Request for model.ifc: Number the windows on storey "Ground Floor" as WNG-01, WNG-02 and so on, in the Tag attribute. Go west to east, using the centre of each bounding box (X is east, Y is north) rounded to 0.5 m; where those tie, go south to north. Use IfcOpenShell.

First a look at what the model holds.

```python
import ifcopenshell
import ifcopenshell.util.element
import ifcopenshell.util.placement

model = ifcopenshell.open("model.ifc")
print(model.schema)
storey = next(s for s in model.by_type("IfcBuildingStorey") if s.Name == "Ground Floor")
windows = [e for e in ifcopenshell.util.element.get_decomposition(storey) if e.is_a("IfcWindow")]
for e in sorted(windows, key=lambda e: e.id()):
    origin = ifcopenshell.util.placement.get_local_placement(e.ObjectPlacement)[:3, 3]
    print(e.id(), e.Tag, e.Name, origin.round(2) + 0.0, sep=" | ")
```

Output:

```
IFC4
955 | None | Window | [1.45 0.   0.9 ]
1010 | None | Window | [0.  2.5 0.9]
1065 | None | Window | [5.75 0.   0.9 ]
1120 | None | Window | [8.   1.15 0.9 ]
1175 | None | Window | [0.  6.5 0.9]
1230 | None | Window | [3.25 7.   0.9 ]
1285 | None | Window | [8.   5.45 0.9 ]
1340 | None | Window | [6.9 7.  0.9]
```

```python
import ifcopenshell
import ifcopenshell.geom
import ifcopenshell.util.element
import ifcopenshell.util.shape

model = ifcopenshell.open("model.ifc")
settings = ifcopenshell.geom.settings()
settings.set("use-world-coords", True)


def centre(element):
    shape = ifcopenshell.geom.create_shape(settings, element)
    return ifcopenshell.util.shape.get_bbox_centroid(shape.geometry)


storey = next(s for s in model.by_type("IfcBuildingStorey") if s.Name == "Ground Floor")
windows = [e for e in ifcopenshell.util.element.get_decomposition(storey) if e.is_a("IfcWindow")]

# Insertion points can sit at a corner or the storey origin, so sort by the geometry (in metres).
centres = {e: centre(e) for e in windows}
windows.sort(key=lambda e: (round(centres[e][0] / 0.5), centres[e][1]))

for i, e in enumerate(windows, start=1):
    number = f"WNG-{i:02d}"
    e.Tag = number
    print(e.id(), number)

model.write("model_v2.ifc")
```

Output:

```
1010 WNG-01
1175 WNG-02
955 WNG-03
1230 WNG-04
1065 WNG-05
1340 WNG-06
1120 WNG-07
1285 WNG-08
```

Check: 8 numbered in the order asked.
